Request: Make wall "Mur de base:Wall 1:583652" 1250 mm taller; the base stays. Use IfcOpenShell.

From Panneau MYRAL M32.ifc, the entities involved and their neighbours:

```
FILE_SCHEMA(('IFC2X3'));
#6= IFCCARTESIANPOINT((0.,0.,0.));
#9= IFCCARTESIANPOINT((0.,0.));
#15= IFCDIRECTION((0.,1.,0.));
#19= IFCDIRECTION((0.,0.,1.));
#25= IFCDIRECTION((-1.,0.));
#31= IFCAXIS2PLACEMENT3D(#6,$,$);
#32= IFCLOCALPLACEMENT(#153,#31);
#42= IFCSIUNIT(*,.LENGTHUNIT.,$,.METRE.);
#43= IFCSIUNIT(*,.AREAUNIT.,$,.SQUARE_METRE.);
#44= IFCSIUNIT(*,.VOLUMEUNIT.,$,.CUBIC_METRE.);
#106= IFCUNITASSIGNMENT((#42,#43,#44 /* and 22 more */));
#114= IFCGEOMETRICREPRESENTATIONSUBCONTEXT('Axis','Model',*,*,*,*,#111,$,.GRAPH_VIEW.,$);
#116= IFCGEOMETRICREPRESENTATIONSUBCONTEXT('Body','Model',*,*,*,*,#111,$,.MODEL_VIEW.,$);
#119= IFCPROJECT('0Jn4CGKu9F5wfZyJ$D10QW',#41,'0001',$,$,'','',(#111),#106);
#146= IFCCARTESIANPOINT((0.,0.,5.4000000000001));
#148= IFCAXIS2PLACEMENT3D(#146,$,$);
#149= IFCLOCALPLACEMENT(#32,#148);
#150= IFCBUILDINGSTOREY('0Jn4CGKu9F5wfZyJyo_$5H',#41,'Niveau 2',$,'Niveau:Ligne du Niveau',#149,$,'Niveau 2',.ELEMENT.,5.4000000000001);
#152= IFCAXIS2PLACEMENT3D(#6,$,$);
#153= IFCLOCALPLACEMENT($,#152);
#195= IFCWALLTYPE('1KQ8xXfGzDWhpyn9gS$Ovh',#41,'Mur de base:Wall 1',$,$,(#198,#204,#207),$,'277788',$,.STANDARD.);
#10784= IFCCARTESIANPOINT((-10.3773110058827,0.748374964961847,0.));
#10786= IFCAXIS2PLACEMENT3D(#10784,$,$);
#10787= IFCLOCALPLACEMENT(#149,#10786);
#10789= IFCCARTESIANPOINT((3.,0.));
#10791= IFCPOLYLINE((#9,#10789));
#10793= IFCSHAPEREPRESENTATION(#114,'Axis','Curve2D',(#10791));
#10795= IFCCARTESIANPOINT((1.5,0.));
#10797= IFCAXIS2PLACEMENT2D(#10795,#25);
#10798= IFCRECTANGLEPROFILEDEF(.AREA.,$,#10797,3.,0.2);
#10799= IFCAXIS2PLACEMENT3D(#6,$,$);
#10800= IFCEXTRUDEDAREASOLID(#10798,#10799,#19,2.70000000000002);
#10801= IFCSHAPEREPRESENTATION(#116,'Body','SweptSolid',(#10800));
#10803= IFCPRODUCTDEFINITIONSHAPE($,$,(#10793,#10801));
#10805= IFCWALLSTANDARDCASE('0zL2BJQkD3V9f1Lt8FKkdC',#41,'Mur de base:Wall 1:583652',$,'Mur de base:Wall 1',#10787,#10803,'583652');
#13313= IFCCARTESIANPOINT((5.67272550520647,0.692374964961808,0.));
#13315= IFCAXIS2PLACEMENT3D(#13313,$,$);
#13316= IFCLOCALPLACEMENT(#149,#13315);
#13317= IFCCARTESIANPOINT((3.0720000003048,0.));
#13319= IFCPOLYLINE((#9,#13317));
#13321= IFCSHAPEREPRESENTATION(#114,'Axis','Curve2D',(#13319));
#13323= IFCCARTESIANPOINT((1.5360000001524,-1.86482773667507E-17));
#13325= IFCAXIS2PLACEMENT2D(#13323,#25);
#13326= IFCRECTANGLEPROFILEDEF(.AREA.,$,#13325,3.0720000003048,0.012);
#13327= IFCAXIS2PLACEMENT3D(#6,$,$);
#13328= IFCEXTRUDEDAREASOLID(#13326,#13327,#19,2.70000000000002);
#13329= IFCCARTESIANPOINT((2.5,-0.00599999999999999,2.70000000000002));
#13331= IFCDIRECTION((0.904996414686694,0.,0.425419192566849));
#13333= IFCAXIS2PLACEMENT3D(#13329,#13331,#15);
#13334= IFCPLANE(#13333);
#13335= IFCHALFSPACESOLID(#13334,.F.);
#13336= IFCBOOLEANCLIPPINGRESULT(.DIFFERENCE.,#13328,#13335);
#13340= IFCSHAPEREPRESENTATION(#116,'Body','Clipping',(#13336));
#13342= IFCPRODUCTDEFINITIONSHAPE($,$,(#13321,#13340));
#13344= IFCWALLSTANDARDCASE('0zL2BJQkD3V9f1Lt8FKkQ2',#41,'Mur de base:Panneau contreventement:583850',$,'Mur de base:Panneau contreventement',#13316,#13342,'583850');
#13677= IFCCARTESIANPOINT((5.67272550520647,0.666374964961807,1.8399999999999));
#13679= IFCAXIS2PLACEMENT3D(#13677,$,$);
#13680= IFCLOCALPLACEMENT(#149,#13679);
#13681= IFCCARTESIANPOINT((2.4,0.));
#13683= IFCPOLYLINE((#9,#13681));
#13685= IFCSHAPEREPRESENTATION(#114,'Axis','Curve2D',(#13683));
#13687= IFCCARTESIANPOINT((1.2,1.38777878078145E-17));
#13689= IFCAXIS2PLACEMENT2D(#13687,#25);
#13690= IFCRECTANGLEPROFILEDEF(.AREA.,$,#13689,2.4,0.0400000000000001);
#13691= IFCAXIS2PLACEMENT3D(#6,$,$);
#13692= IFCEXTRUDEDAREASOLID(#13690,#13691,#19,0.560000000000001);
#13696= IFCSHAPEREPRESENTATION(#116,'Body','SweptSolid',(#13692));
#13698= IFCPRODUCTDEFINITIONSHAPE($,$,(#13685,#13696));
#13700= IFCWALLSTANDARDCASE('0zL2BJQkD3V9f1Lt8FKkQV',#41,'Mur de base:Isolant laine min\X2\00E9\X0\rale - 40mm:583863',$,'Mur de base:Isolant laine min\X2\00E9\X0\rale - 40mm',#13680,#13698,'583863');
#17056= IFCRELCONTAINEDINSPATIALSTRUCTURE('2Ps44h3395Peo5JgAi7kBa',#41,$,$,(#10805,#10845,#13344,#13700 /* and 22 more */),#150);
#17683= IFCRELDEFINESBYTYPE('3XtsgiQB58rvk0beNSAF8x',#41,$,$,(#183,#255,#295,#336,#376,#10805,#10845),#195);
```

```python
import ifcopenshell
import ifcopenshell.geom
import ifcopenshell.util.representation
import ifcopenshell.util.shape

model = ifcopenshell.open("Panneau MYRAL M32.ifc")
settings = ifcopenshell.geom.settings()


def volume(element):
    """Net volume in cubic metres, openings subtracted."""
    shape = ifcopenshell.geom.create_shape(settings, element)
    return ifcopenshell.util.shape.get_volume(shape.geometry)


wall = model.by_guid("0zL2BJQkD3V9f1Lt8FKkdC")
before = volume(wall)

body = ifcopenshell.util.representation.get_representation(wall, "Model", "Body")
solid = body.Items[0]
old_height = solid.Depth
solid.Depth += 1.25
after = volume(wall)

print(f"height {old_height:g} -> {solid.Depth:g}, volume {before:.3f} -> {after:.3f} m3")

model.write("Panneau MYRAL M32-out.ifc")
```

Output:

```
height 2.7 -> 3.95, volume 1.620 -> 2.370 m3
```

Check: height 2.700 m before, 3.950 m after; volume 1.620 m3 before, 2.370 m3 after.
